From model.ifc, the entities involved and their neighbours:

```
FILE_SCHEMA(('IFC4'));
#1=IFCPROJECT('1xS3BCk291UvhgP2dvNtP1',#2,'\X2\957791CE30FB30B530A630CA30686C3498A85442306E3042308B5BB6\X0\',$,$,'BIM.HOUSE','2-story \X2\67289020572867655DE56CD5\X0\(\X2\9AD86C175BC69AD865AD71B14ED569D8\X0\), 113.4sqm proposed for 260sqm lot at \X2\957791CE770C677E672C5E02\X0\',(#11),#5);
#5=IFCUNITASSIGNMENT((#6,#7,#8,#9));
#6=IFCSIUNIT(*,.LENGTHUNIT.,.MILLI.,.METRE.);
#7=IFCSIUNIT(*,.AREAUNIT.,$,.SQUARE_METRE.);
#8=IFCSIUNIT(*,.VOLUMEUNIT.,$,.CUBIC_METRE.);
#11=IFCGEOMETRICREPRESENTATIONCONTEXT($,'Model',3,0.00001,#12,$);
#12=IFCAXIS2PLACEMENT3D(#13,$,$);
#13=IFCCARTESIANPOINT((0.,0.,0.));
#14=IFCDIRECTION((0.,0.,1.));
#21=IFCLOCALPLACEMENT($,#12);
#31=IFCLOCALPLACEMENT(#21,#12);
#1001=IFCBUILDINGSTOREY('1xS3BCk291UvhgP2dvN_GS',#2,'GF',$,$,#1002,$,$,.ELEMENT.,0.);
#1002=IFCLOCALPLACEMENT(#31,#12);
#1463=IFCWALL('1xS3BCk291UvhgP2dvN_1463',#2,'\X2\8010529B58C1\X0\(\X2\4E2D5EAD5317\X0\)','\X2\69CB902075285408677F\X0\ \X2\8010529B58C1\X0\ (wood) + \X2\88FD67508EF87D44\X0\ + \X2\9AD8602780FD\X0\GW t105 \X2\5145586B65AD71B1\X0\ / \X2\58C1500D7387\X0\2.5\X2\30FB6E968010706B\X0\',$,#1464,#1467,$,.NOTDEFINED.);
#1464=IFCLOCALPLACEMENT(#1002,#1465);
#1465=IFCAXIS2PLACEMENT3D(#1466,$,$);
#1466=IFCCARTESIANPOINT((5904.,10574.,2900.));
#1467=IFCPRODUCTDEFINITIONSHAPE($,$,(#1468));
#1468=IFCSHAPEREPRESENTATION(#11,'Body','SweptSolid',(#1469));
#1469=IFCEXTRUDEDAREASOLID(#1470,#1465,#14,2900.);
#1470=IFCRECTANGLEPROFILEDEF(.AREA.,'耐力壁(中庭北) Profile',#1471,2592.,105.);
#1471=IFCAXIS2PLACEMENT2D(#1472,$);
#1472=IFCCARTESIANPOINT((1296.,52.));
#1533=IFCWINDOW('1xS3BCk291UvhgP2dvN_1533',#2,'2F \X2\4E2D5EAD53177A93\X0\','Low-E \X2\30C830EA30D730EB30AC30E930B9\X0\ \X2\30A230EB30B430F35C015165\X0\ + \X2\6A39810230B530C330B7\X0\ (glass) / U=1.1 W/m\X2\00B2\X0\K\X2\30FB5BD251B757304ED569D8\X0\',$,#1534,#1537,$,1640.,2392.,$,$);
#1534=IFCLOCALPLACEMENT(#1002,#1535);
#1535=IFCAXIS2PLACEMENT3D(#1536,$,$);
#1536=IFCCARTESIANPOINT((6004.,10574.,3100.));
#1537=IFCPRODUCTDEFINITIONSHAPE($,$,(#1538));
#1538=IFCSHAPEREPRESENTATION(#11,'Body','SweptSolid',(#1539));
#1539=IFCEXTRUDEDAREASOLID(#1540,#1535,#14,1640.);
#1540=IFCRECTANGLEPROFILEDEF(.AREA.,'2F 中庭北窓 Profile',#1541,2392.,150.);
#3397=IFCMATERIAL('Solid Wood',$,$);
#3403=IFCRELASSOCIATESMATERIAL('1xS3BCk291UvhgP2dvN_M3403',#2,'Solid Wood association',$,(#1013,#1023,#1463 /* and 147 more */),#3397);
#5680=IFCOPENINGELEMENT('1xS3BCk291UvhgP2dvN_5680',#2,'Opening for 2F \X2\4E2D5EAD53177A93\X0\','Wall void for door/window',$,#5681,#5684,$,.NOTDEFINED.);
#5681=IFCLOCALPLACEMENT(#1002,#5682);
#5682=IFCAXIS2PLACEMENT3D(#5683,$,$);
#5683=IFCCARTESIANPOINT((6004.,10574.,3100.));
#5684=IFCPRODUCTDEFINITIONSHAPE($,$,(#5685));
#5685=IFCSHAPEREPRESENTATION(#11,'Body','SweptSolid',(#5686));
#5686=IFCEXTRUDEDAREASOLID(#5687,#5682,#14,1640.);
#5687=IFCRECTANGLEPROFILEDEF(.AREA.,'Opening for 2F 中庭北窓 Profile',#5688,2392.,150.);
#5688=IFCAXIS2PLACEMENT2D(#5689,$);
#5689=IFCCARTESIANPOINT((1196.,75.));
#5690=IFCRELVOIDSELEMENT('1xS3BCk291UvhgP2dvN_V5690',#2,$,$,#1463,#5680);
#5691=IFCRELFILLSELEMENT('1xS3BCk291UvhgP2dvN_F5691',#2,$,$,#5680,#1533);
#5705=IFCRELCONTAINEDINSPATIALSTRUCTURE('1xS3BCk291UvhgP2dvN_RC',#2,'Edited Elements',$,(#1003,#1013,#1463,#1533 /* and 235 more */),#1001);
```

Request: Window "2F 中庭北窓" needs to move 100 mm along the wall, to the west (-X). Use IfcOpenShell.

```python
import ifcopenshell
import ifcopenshell.api.geometry
import ifcopenshell.util.placement
import ifcopenshell.util.unit

model = ifcopenshell.open("model.ifc")
unit_scale = ifcopenshell.util.unit.calculate_unit_scale(model)

window = model.by_id(1533)
opening = window.FillsVoids[0].RelatingOpeningElement
wall = opening.VoidsElements[0].RelatingBuildingElement

wall_matrix = ifcopenshell.util.placement.get_local_placement(wall.ObjectPlacement)
shift = wall_matrix[:3, 0] * -0.1 / unit_scale
before = ifcopenshell.util.placement.get_local_placement(window.ObjectPlacement)[:3, 3].copy()

# The window is not placed relative to its opening, so move both.
for product in (opening, window):
    matrix = ifcopenshell.util.placement.get_local_placement(product.ObjectPlacement)
    matrix[:3, 3] += shift
    ifcopenshell.api.geometry.edit_object_placement(model, product=product, matrix=matrix, is_si=False)

after = ifcopenshell.util.placement.get_local_placement(window.ObjectPlacement)[:3, 3]
print("window moved by", (after - before).round(3) + 0.0)

model.write("model-out.ifc")
```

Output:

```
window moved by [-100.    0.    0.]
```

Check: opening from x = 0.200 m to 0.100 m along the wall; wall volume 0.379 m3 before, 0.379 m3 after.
